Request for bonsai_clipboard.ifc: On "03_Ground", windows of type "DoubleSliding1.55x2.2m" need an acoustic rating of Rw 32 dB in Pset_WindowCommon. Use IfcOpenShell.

First a look at what the model holds.

```python
import ifcopenshell
import ifcopenshell.util.element

model = ifcopenshell.open("bonsai_clipboard.ifc")
print(model.schema)
storey = next(s for s in model.by_type("IfcBuildingStorey") if s.Name == "03_Ground")
windows = [e for e in ifcopenshell.util.element.get_decomposition(storey) if e.is_a("IfcWindow")]
seen = {}
for e in windows:
    element_type = ifcopenshell.util.element.get_type(e)
    key = (element_type.Name if element_type != e and element_type else None, ifcopenshell.util.element.get_pset(e, "Pset_WindowCommon", "AcousticRating"))
    seen[key] = seen.get(key, 0) + 1
for (name, value), count in sorted(seen.items(), key=str):
    print(count, "x", name, "|", value)
```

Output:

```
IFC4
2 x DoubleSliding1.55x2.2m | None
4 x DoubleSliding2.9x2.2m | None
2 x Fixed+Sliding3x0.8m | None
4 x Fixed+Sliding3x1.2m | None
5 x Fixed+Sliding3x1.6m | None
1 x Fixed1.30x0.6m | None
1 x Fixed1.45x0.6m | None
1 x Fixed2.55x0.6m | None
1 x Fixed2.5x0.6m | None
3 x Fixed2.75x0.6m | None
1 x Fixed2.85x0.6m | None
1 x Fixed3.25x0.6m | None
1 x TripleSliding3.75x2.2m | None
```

```python
import ifcopenshell
import ifcopenshell.api.pset
import ifcopenshell.util.element

model = ifcopenshell.open("bonsai_clipboard.ifc")

storey = next(s for s in model.by_type("IfcBuildingStorey") if s.Name == "03_Ground")
windows = [e for e in ifcopenshell.util.element.get_decomposition(storey) if e.is_a("IfcWindow")]

count = 0
for e in windows:
    element_type = ifcopenshell.util.element.get_type(e)
    if element_type in (None, e) or element_type.Name != "DoubleSliding1.55x2.2m":
        continue
    # add_pset returns the element's existing set when there is one.
    pset = ifcopenshell.api.pset.add_pset(model, product=e, name="Pset_WindowCommon")
    ifcopenshell.api.pset.edit_pset(model, pset=pset, properties={"AcousticRating": "Rw 32 dB"})
    count += 1

print(count, "windows updated")

model.write("bonsai_clipboard_edited.ifc")
```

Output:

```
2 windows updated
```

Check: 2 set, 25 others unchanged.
